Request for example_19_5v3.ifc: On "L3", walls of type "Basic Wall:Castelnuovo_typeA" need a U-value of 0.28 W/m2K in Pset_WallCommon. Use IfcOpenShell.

First a look at what the model holds.

```python
import ifcopenshell
import ifcopenshell.util.element

model = ifcopenshell.open("example_19_5v3.ifc")
print(model.schema)
storey = next(s for s in model.by_type("IfcBuildingStorey") if s.Name == "L3")
walls = [e for e in ifcopenshell.util.element.get_decomposition(storey) if e.is_a("IfcWall")]
seen = {}
for e in walls:
    element_type = ifcopenshell.util.element.get_type(e)
    key = (element_type.Name if element_type != e and element_type else None, ifcopenshell.util.element.get_pset(e, "Pset_WallCommon", "ThermalTransmittance"))
    seen[key] = seen.get(key, 0) + 1
for (name, value), count in sorted(seen.items(), key=str):
    print(count, "x", name, "|", value)
```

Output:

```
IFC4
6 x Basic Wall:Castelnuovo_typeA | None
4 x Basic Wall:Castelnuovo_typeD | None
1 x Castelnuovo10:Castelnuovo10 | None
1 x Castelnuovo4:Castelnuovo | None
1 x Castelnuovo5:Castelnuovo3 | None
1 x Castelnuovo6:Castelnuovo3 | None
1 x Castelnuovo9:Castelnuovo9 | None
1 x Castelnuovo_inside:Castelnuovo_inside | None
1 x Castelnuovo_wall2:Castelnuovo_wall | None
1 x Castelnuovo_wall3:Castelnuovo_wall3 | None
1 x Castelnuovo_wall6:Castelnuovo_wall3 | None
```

```python
import ifcopenshell
import ifcopenshell.api.pset
import ifcopenshell.util.element

model = ifcopenshell.open("example_19_5v3.ifc")

storey = next(s for s in model.by_type("IfcBuildingStorey") if s.Name == "L3")
walls = [e for e in ifcopenshell.util.element.get_decomposition(storey) if e.is_a("IfcWall")]

count = 0
for e in walls:
    element_type = ifcopenshell.util.element.get_type(e)
    if element_type in (None, e) or element_type.Name != "Basic Wall:Castelnuovo_typeA":
        continue
    # add_pset returns the element's existing set when there is one.
    pset = ifcopenshell.api.pset.add_pset(model, product=e, name="Pset_WallCommon")
    ifcopenshell.api.pset.edit_pset(model, pset=pset, properties={"ThermalTransmittance": 0.28})
    count += 1

print(count, "walls updated")

model.write("example_19_5v3-out.ifc")
```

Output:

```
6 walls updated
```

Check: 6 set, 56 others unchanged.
